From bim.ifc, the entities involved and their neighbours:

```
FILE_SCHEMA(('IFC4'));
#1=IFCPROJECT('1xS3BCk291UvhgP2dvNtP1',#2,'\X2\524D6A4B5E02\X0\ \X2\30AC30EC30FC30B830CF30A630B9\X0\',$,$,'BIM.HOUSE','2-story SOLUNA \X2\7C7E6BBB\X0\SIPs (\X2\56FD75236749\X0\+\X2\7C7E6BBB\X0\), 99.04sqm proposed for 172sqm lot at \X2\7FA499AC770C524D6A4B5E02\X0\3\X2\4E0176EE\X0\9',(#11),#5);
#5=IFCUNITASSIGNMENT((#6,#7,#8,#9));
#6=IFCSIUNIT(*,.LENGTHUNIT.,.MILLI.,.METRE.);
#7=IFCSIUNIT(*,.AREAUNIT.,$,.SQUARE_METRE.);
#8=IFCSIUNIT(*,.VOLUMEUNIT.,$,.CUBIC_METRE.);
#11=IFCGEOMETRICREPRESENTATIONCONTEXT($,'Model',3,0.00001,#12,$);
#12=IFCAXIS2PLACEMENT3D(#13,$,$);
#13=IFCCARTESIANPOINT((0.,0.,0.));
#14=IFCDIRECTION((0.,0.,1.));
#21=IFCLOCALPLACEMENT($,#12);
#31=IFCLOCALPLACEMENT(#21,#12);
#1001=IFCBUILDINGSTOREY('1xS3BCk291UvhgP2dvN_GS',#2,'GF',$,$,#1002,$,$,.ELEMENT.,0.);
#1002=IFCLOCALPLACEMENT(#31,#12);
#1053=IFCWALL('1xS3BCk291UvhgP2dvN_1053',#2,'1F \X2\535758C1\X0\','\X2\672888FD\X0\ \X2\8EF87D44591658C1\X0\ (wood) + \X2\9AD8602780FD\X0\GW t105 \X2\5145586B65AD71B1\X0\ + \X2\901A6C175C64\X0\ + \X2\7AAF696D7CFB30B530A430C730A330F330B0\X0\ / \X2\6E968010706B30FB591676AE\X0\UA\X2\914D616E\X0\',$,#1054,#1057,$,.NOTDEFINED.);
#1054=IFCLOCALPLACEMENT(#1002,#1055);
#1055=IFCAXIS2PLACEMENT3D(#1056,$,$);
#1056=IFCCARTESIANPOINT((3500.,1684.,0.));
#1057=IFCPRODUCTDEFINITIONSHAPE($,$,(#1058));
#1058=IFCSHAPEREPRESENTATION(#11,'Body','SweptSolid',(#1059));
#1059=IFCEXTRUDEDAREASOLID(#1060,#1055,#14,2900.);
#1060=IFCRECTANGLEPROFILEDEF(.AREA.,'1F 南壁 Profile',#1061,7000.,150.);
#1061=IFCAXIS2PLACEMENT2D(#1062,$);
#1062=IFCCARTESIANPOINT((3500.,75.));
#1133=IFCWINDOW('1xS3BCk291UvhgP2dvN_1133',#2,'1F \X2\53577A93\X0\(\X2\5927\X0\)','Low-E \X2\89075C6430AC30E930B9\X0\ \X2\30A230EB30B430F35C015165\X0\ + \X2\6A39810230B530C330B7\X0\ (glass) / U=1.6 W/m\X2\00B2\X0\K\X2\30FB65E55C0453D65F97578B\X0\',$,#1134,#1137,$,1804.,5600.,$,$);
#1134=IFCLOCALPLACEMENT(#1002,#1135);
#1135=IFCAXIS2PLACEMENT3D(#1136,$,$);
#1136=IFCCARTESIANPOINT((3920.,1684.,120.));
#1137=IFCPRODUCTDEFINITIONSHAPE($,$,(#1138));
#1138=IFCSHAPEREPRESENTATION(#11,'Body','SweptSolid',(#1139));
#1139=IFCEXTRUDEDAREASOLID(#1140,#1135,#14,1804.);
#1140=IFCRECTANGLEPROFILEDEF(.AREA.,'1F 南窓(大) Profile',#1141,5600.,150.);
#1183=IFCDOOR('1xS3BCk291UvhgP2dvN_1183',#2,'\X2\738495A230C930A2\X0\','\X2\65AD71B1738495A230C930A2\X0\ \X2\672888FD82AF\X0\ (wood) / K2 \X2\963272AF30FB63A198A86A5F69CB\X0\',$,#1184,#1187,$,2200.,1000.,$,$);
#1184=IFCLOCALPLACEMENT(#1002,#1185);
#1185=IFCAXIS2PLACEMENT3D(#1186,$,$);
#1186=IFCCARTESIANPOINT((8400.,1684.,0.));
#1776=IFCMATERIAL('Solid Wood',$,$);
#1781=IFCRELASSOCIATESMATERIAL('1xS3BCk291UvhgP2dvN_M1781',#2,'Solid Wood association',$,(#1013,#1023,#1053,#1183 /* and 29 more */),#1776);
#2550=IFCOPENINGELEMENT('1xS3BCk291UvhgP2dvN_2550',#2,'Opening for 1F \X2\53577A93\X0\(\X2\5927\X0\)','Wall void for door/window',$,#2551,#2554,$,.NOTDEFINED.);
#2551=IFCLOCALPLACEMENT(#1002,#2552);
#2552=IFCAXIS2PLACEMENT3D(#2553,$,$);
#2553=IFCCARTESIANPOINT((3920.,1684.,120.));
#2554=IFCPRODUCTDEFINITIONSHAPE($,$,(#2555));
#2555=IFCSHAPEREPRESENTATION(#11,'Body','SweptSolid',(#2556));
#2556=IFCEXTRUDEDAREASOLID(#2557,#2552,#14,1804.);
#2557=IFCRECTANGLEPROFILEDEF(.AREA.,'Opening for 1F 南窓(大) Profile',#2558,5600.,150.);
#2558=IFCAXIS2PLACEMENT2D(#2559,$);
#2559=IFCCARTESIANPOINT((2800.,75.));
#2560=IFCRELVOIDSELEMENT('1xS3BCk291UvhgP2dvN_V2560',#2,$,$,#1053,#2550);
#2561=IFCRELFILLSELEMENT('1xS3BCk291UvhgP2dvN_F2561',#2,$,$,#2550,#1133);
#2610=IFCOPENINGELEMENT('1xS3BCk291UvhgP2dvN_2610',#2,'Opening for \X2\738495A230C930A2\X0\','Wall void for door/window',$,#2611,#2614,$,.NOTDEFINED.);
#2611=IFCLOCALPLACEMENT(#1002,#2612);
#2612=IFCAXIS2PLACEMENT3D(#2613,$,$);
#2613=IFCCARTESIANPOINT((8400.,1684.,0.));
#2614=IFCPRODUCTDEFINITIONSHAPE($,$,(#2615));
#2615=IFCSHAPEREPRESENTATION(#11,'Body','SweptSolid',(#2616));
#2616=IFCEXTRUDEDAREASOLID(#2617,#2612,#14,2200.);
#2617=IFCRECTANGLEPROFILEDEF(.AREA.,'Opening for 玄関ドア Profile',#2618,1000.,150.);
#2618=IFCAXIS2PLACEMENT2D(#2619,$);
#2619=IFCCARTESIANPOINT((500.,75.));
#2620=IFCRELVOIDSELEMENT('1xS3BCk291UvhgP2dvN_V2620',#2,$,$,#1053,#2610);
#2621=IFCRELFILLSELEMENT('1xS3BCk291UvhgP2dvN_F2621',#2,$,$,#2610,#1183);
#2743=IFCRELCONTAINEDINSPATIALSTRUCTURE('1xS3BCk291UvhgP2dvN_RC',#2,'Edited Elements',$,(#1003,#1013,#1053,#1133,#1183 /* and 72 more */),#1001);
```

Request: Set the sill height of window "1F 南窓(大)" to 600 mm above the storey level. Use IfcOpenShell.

```python
import numpy as np
import ifcopenshell
import ifcopenshell.api.geometry
import ifcopenshell.geom
import ifcopenshell.util.element
import ifcopenshell.util.placement
import ifcopenshell.util.shape
import ifcopenshell.util.unit

model = ifcopenshell.open("bim.ifc")
unit_scale = ifcopenshell.util.unit.calculate_unit_scale(model)

window = model.by_guid("1xS3BCk291UvhgP2dvN_1133")
opening = window.FillsVoids[0].RelatingOpeningElement
storey = ifcopenshell.util.element.get_container(window, ifc_class="IfcBuildingStorey")
level = ifcopenshell.util.placement.get_local_placement(storey.ObjectPlacement)[2, 3]

# The opening's origin need not be at the sill, so measure its lowest point.
shape = ifcopenshell.geom.create_shape(ifcopenshell.geom.settings(), opening)
bottom = ifcopenshell.util.shape.get_shape_bottom_elevation(shape, shape.geometry) / unit_scale
dz = level + 600.0 - bottom

shift = np.array([0.0, 0.0, dz])
# The window is not placed relative to its opening, so move both.
for product in (opening, window):
    matrix = ifcopenshell.util.placement.get_local_placement(product.ObjectPlacement)
    matrix[:3, 3] += shift
    ifcopenshell.api.geometry.edit_object_placement(model, product=product, matrix=matrix, is_si=False)

print(f"moved by {dz * unit_scale:+.3f} m")

model.write("bim_edited.ifc")
```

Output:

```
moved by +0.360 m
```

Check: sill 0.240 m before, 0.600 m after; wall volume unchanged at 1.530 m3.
